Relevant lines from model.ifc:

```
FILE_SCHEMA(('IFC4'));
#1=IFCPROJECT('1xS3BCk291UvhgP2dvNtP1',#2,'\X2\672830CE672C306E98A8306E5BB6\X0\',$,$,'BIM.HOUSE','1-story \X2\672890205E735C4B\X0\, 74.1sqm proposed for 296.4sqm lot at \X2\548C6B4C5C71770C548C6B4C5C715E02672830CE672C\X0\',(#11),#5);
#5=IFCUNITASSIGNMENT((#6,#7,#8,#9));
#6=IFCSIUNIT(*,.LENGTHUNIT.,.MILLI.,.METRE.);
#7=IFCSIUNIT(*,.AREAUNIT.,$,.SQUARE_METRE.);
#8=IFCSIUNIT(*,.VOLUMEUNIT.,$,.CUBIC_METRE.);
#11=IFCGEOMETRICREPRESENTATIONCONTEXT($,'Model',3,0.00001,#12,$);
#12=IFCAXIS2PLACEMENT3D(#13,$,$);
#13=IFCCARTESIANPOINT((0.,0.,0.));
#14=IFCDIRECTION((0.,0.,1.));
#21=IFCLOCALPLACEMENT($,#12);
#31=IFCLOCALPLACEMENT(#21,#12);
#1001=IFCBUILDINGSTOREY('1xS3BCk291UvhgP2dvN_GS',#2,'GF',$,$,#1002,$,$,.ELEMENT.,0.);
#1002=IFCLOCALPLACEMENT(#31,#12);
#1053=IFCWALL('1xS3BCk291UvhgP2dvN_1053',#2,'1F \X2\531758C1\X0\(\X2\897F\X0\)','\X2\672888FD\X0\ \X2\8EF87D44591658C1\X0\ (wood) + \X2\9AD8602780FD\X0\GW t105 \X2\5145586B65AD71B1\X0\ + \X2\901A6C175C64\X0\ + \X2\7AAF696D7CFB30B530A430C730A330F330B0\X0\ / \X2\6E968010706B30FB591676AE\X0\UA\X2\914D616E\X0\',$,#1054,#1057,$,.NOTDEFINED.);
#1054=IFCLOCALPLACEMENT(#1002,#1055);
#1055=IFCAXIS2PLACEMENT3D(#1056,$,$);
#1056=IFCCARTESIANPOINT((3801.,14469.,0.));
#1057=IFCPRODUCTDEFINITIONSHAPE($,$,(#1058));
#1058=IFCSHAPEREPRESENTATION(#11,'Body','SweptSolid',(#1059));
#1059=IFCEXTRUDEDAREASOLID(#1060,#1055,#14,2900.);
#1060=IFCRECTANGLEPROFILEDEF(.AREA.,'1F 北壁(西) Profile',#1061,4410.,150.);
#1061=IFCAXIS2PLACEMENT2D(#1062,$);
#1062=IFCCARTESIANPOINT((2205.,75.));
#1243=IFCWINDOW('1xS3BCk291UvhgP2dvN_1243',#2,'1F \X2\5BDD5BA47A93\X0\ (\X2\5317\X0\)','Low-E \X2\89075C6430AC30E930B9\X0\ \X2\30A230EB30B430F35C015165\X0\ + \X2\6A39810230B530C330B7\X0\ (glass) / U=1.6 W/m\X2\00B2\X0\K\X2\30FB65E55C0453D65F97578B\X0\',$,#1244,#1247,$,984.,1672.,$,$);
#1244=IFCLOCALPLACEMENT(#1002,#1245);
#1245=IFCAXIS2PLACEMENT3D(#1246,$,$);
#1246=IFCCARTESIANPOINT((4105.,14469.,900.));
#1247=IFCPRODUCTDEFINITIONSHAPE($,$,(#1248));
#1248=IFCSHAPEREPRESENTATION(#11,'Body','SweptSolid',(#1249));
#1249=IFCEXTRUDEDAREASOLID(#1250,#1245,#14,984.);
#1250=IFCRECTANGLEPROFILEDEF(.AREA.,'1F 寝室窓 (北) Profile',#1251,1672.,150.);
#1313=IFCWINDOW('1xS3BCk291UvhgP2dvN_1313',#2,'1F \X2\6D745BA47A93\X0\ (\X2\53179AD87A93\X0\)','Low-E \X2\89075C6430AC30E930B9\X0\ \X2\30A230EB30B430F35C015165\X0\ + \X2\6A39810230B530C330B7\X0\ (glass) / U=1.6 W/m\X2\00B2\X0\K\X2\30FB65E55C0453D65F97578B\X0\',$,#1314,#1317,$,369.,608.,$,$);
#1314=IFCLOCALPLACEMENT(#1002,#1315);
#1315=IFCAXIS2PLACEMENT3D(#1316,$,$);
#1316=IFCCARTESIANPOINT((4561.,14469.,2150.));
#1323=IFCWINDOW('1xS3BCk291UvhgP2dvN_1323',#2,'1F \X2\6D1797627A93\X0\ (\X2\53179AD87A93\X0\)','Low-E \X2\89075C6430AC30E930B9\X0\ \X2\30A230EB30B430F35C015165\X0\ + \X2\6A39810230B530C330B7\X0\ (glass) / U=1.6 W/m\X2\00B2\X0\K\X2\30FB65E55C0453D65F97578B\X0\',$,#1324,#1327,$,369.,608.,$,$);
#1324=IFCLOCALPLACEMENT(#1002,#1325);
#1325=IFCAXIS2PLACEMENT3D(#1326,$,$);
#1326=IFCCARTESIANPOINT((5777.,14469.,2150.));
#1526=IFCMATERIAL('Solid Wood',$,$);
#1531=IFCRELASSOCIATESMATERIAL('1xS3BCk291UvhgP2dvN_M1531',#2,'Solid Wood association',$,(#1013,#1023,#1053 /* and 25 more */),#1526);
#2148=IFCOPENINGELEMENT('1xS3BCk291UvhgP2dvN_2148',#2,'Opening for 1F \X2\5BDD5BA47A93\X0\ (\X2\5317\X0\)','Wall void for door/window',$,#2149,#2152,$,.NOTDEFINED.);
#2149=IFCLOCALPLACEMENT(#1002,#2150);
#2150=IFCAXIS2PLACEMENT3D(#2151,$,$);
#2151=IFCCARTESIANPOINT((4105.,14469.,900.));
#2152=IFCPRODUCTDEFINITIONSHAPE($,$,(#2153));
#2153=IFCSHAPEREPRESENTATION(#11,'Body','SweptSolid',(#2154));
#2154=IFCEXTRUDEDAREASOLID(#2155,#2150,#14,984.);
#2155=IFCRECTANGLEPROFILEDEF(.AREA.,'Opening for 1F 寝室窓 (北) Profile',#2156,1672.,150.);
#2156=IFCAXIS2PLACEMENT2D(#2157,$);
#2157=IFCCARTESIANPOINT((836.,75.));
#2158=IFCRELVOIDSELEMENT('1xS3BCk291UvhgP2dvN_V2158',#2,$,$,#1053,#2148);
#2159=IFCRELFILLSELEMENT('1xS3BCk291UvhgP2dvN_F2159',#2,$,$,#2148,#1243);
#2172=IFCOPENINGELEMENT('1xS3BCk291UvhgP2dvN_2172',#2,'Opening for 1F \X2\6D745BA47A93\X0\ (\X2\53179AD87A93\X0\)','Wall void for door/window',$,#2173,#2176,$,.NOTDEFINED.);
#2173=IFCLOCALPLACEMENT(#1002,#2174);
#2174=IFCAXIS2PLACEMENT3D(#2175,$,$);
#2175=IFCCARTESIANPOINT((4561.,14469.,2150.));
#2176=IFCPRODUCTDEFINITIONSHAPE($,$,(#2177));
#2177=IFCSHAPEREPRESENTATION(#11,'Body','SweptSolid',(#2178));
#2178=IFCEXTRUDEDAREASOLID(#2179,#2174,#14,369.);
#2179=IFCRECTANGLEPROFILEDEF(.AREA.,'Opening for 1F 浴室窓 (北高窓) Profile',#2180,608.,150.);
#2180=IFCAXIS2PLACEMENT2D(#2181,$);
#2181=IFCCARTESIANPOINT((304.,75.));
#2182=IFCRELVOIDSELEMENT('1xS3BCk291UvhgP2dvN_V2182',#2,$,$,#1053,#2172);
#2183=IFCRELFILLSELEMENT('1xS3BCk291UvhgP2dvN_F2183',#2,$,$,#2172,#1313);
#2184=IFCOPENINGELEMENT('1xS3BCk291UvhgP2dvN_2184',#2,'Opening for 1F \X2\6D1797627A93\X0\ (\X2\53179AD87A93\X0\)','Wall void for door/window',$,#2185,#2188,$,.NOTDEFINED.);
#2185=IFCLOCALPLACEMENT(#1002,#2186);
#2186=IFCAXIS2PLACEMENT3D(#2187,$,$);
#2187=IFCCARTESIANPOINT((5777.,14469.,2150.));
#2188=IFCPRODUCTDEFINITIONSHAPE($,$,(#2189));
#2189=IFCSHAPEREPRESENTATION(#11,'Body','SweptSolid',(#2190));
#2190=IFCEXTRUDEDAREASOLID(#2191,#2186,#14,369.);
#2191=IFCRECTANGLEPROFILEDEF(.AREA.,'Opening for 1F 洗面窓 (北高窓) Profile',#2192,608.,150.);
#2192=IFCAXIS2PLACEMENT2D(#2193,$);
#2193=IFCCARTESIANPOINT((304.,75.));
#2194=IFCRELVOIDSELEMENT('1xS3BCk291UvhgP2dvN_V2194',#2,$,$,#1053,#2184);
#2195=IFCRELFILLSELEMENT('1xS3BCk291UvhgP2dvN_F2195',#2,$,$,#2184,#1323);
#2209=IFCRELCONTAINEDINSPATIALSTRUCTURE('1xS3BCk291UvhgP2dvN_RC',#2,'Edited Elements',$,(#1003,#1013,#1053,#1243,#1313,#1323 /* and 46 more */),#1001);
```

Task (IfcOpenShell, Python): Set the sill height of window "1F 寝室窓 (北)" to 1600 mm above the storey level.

```python
import numpy as np
import ifcopenshell
import ifcopenshell.api.geometry
import ifcopenshell.geom
import ifcopenshell.util.element
import ifcopenshell.util.placement
import ifcopenshell.util.shape
import ifcopenshell.util.unit

model = ifcopenshell.open("model.ifc")
unit_scale = ifcopenshell.util.unit.calculate_unit_scale(model)

window = model.by_guid("1xS3BCk291UvhgP2dvN_1243")
opening = window.FillsVoids[0].RelatingOpeningElement
storey = ifcopenshell.util.element.get_container(window, ifc_class="IfcBuildingStorey")
level = ifcopenshell.util.placement.get_local_placement(storey.ObjectPlacement)[2, 3]

# The opening's origin need not be at the sill, so measure its lowest point.
shape = ifcopenshell.geom.create_shape(ifcopenshell.geom.settings(), opening)
bottom = ifcopenshell.util.shape.get_shape_bottom_elevation(shape, shape.geometry) / unit_scale
dz = level + 1.6 / unit_scale - bottom

shift = np.array([0.0, 0.0, dz])
# The window is not placed relative to its opening, so move both.
for product in (opening, window):
    matrix = ifcopenshell.util.placement.get_local_placement(product.ObjectPlacement)
    matrix[:3, 3] += shift
    ifcopenshell.api.geometry.edit_object_placement(model, product=product, matrix=matrix, is_si=False)

print(f"moved by {dz * unit_scale:+.3f} m")

model.write("model_rev.ifc")
```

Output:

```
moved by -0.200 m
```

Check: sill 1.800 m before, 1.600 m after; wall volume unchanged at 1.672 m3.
